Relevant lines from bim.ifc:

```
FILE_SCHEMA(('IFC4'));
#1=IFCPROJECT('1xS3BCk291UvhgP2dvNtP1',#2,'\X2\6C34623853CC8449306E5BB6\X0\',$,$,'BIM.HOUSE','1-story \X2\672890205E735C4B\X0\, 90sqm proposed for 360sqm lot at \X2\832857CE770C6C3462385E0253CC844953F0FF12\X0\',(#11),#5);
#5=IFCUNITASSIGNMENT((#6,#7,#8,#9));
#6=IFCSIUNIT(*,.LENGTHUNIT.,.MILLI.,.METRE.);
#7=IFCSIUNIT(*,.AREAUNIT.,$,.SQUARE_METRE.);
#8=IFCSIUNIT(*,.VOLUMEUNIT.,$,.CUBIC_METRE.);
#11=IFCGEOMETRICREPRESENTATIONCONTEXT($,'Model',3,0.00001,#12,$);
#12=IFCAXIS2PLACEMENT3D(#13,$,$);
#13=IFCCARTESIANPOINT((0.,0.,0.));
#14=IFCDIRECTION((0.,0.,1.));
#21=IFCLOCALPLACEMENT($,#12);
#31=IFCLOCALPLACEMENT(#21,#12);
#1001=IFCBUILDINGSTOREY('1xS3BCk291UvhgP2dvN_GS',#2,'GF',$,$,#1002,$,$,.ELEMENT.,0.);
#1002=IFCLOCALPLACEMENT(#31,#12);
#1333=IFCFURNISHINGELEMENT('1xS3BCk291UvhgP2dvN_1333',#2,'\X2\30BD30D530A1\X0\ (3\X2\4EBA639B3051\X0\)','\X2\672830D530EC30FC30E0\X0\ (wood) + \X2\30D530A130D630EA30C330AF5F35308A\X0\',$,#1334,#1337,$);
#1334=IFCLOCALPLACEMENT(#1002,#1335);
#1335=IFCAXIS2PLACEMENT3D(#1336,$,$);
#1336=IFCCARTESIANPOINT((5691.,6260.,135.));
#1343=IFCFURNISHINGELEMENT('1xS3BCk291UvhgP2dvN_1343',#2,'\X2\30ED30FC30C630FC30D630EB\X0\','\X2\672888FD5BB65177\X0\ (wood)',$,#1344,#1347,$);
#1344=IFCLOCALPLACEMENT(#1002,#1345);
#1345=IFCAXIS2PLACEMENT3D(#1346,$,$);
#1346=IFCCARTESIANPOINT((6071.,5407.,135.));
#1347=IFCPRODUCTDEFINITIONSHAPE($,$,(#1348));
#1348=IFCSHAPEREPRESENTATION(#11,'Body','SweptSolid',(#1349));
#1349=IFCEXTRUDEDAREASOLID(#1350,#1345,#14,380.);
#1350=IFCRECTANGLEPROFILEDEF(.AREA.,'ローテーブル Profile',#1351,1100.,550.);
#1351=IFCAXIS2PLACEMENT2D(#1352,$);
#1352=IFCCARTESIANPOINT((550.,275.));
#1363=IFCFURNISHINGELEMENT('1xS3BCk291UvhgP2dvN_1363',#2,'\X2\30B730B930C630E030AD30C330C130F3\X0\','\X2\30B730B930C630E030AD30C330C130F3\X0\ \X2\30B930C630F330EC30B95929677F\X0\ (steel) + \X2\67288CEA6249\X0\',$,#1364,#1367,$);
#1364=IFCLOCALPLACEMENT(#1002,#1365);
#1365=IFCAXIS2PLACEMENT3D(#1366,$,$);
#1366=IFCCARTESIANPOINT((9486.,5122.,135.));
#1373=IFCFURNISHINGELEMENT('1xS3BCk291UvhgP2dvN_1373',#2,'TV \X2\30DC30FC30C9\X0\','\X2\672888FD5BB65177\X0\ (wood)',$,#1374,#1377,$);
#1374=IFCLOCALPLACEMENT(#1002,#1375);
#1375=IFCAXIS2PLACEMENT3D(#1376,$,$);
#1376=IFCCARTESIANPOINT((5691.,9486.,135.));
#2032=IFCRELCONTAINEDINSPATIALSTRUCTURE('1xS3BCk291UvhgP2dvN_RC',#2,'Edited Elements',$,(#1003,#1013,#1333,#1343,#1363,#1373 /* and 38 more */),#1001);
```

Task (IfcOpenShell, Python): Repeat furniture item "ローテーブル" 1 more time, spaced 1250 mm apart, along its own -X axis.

```python
import ifcopenshell
import ifcopenshell.api.geometry
import ifcopenshell.api.root
import ifcopenshell.util.element
import ifcopenshell.util.placement
import ifcopenshell.util.unit

model = ifcopenshell.open("bim.ifc")
unit_scale = ifcopenshell.util.unit.calculate_unit_scale(model)


def reuse_history(source, copy):
    """copy_class also copies each property set's owner history, people and application; keep the originals."""
    for rel in copy.IsDefinedBy:
        if rel.is_a("IfcRelDefinesByProperties") and (history := rel.RelatingPropertyDefinition.OwnerHistory):
            rel.RelatingPropertyDefinition.OwnerHistory = source.OwnerHistory
            ifcopenshell.util.element.remove_deep2(model, history)


source = model.by_guid("1xS3BCk291UvhgP2dvN_1343")
base = ifcopenshell.util.placement.get_local_placement(source.ObjectPlacement)
step = -base[:3, 0] * 1.25 / unit_scale

for i in range(1, 2):
    copy = ifcopenshell.api.root.copy_class(model, product=source)
    copy.Representation = ifcopenshell.util.element.copy_deep(
        model, source.Representation, exclude=["IfcGeometricRepresentationContext", "IfcRepresentationMap"]
    )
    reuse_history(source, copy)
    matrix = base.copy()
    matrix[:3, 3] += i * step
    print("added at", matrix[:3, 3].round(3) + 0.0)
    ifcopenshell.api.geometry.edit_object_placement(model, product=copy, matrix=matrix, is_si=False)

model.write("bim_v2.ifc")
```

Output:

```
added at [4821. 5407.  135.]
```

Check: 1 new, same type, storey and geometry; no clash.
